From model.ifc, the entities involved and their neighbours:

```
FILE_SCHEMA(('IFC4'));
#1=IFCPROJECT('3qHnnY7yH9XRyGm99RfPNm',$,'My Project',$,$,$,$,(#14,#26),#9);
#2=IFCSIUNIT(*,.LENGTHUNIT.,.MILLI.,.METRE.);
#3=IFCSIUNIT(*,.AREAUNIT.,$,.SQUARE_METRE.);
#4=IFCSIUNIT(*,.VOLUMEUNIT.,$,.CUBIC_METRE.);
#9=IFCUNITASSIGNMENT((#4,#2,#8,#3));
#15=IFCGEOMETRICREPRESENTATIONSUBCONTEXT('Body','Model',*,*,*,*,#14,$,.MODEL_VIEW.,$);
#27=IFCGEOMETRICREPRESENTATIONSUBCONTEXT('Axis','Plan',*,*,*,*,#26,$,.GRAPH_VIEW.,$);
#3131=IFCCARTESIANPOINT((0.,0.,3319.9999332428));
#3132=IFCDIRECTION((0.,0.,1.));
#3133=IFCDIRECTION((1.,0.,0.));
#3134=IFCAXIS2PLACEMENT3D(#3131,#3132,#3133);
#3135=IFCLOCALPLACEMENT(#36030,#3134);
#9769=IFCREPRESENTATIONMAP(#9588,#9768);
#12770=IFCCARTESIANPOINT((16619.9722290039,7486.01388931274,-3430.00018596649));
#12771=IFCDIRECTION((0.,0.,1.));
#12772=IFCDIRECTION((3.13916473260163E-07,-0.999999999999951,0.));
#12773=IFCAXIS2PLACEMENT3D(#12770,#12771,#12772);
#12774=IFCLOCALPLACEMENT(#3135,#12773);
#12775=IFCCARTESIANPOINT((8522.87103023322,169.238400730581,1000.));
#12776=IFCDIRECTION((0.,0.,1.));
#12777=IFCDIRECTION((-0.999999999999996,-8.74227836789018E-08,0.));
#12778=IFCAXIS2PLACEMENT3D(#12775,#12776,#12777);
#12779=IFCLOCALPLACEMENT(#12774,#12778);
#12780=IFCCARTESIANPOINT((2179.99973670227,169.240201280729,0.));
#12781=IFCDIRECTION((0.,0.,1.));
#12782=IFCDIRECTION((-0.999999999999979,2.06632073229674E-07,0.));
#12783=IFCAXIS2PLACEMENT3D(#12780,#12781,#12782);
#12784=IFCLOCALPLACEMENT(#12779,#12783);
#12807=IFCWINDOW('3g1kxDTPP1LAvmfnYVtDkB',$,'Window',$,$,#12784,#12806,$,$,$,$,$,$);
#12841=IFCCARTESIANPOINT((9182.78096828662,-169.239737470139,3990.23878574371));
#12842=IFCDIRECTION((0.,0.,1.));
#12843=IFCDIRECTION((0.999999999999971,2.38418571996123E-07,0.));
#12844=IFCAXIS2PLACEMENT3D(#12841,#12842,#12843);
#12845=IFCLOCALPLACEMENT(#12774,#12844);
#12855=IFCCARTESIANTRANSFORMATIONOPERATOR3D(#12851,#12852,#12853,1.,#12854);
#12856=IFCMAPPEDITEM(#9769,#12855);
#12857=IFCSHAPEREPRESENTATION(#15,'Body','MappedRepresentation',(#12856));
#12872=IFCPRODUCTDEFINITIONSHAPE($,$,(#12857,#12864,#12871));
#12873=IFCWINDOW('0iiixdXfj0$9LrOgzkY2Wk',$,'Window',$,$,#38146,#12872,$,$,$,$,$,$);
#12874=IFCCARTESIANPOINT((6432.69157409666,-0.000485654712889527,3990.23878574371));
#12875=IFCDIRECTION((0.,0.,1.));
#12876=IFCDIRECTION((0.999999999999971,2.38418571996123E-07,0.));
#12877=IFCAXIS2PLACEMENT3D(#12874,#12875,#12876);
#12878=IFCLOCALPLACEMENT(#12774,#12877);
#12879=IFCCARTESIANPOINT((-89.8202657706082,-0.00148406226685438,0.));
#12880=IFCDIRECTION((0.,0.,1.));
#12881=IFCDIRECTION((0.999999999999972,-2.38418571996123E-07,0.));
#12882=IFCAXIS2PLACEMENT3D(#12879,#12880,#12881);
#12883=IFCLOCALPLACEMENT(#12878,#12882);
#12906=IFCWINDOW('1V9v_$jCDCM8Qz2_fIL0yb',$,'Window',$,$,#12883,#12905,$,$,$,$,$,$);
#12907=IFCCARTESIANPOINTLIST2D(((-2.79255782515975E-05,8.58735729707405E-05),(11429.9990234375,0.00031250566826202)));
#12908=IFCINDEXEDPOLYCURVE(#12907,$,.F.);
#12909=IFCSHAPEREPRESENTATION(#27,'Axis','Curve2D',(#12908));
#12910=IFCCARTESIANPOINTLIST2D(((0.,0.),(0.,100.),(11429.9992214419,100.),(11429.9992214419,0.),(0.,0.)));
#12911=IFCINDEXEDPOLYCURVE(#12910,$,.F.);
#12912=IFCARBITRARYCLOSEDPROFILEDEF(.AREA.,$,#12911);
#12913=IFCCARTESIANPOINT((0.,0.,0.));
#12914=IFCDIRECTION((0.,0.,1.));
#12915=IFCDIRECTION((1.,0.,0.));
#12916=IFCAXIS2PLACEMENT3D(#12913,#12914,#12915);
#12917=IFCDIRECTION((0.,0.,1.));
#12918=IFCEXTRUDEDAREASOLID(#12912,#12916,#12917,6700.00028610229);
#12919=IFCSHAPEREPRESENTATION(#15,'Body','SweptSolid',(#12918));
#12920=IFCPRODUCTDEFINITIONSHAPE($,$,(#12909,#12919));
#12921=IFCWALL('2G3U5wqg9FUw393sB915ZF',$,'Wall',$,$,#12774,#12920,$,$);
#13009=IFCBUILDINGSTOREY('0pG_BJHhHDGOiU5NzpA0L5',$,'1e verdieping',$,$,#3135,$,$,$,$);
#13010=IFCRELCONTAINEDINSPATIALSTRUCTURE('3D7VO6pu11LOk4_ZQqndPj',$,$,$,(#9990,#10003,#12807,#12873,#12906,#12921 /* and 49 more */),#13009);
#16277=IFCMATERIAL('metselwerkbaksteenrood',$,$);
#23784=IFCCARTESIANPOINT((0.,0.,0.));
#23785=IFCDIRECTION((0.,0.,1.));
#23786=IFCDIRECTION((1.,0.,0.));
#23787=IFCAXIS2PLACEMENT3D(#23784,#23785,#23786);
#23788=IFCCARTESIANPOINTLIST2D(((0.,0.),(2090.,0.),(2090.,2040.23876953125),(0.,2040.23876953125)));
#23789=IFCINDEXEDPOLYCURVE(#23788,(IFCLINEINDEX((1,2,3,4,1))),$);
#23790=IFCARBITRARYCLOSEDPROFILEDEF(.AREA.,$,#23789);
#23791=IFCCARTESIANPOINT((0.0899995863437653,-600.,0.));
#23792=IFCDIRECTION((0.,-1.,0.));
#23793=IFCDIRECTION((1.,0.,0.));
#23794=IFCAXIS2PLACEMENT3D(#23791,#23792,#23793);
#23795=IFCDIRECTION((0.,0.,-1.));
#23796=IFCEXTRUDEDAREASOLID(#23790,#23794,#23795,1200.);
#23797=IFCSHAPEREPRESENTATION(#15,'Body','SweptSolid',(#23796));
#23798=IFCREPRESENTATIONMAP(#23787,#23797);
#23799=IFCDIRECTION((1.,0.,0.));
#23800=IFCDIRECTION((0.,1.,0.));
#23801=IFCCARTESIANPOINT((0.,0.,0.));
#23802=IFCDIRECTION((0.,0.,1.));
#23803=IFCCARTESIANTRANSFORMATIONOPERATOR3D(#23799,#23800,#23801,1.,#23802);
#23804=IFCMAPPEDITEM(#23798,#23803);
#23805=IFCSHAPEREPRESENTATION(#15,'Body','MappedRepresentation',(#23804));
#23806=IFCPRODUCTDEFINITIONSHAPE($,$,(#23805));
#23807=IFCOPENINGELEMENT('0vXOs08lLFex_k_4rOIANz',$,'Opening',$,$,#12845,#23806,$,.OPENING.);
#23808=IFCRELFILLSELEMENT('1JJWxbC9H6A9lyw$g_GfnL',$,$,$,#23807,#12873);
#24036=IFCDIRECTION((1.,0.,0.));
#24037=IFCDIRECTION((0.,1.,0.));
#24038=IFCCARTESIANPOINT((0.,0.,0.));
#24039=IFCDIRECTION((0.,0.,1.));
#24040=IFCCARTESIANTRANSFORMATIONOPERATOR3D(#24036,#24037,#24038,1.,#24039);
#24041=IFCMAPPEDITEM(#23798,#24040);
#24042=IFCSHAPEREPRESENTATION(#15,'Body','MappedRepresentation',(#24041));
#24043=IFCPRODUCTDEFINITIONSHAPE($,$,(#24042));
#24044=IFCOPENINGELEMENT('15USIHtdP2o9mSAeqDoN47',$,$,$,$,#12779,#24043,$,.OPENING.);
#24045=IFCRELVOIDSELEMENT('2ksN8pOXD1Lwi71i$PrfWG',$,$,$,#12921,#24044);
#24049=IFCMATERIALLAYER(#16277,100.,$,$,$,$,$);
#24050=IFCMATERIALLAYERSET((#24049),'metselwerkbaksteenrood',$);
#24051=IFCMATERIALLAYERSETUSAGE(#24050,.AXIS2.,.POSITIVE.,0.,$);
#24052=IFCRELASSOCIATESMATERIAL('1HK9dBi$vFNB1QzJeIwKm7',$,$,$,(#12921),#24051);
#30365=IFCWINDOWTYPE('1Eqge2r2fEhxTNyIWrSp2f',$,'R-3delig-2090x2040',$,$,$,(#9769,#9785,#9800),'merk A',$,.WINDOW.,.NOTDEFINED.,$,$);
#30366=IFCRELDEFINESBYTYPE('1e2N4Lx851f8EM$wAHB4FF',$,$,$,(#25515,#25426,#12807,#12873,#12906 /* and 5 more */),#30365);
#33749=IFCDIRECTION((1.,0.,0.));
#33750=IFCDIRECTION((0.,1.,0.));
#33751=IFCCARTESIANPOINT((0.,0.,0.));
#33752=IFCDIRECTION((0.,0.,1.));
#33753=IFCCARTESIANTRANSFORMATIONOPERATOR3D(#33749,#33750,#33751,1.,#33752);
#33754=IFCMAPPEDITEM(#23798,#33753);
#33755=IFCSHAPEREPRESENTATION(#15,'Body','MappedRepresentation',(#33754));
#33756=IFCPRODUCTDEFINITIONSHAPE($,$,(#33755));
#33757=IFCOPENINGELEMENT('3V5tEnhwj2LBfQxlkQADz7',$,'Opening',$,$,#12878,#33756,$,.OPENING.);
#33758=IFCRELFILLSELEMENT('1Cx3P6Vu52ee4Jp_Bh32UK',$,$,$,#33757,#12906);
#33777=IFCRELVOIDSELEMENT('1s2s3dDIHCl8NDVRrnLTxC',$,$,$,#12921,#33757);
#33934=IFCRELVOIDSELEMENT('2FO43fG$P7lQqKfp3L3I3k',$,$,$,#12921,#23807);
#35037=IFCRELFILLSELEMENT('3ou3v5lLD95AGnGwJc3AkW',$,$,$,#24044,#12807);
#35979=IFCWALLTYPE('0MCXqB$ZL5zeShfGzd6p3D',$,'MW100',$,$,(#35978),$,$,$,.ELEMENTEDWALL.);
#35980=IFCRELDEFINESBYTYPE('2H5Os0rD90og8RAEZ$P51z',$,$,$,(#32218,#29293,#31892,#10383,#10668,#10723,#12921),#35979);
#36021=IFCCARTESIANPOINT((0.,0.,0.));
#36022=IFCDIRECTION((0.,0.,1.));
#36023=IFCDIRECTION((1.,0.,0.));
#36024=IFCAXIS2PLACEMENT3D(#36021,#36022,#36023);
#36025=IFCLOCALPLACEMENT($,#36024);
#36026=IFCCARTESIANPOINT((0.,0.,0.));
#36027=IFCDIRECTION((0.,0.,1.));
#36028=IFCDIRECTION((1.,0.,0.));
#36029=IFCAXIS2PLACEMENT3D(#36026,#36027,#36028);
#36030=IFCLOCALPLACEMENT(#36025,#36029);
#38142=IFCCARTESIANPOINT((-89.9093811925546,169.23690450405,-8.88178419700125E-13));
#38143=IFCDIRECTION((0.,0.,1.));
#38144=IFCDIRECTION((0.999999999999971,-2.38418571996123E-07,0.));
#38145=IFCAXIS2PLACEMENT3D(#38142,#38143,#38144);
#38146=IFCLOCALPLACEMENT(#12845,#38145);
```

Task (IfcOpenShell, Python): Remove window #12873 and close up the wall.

```python
import ifcopenshell
import ifcopenshell.api.feature
import ifcopenshell.api.root
import ifcopenshell.geom
import ifcopenshell.util.shape

model = ifcopenshell.open("model.ifc")
settings = ifcopenshell.geom.settings()


def volume(element):
    """Net volume in cubic metres, openings subtracted."""
    shape = ifcopenshell.geom.create_shape(settings, element)
    return ifcopenshell.util.shape.get_volume(shape.geometry)


window = model.by_id(12873)
opening = window.FillsVoids[0].RelatingOpeningElement
wall = opening.VoidsElements[0].RelatingBuildingElement
before = volume(wall)

ifcopenshell.api.root.remove_product(model, product=window)
ifcopenshell.api.feature.remove_feature(model, feature=opening)

after = volume(wall)

print(f"wall volume {before:.3f} -> {after:.3f} m3")

model.write("model_updated.ifc")
```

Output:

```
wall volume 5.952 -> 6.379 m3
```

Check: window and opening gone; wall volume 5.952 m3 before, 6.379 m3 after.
